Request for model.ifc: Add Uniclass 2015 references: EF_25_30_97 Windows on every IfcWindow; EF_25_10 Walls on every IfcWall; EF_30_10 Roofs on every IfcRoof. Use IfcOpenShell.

First a look at what the model holds.

```python
import ifcopenshell

model = ifcopenshell.open("model.ifc")
print(model.schema)
print("classifications:", [c.Name for c in model.by_type("IfcClassification")])
for ifc_class in ("IfcDoor", "IfcRoof", "IfcStair", "IfcWall", "IfcWindow"):
    print(ifc_class, len(model.by_type(ifc_class)))
```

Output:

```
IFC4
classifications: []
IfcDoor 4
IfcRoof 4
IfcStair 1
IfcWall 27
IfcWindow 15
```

```python
import ifcopenshell
import ifcopenshell.api.classification

model = ifcopenshell.open("model.ifc")

system = ifcopenshell.api.classification.add_classification(model, classification="Uniclass 2015")

codes = {
    "IfcWindow": ("EF_25_30_97", "Windows"),
    "IfcWall": ("EF_25_10", "Walls"),
    "IfcRoof": ("EF_30_10", "Roofs"),
}
for ifc_class, (code, name) in codes.items():
    products = model.by_type(ifc_class)
    ifcopenshell.api.classification.add_reference(
        model, products=products, classification=system, identification=code, name=name
    )
    print(code, len(products))

model.write("model_updated.ifc")
```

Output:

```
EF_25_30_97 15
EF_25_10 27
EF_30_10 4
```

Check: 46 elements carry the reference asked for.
